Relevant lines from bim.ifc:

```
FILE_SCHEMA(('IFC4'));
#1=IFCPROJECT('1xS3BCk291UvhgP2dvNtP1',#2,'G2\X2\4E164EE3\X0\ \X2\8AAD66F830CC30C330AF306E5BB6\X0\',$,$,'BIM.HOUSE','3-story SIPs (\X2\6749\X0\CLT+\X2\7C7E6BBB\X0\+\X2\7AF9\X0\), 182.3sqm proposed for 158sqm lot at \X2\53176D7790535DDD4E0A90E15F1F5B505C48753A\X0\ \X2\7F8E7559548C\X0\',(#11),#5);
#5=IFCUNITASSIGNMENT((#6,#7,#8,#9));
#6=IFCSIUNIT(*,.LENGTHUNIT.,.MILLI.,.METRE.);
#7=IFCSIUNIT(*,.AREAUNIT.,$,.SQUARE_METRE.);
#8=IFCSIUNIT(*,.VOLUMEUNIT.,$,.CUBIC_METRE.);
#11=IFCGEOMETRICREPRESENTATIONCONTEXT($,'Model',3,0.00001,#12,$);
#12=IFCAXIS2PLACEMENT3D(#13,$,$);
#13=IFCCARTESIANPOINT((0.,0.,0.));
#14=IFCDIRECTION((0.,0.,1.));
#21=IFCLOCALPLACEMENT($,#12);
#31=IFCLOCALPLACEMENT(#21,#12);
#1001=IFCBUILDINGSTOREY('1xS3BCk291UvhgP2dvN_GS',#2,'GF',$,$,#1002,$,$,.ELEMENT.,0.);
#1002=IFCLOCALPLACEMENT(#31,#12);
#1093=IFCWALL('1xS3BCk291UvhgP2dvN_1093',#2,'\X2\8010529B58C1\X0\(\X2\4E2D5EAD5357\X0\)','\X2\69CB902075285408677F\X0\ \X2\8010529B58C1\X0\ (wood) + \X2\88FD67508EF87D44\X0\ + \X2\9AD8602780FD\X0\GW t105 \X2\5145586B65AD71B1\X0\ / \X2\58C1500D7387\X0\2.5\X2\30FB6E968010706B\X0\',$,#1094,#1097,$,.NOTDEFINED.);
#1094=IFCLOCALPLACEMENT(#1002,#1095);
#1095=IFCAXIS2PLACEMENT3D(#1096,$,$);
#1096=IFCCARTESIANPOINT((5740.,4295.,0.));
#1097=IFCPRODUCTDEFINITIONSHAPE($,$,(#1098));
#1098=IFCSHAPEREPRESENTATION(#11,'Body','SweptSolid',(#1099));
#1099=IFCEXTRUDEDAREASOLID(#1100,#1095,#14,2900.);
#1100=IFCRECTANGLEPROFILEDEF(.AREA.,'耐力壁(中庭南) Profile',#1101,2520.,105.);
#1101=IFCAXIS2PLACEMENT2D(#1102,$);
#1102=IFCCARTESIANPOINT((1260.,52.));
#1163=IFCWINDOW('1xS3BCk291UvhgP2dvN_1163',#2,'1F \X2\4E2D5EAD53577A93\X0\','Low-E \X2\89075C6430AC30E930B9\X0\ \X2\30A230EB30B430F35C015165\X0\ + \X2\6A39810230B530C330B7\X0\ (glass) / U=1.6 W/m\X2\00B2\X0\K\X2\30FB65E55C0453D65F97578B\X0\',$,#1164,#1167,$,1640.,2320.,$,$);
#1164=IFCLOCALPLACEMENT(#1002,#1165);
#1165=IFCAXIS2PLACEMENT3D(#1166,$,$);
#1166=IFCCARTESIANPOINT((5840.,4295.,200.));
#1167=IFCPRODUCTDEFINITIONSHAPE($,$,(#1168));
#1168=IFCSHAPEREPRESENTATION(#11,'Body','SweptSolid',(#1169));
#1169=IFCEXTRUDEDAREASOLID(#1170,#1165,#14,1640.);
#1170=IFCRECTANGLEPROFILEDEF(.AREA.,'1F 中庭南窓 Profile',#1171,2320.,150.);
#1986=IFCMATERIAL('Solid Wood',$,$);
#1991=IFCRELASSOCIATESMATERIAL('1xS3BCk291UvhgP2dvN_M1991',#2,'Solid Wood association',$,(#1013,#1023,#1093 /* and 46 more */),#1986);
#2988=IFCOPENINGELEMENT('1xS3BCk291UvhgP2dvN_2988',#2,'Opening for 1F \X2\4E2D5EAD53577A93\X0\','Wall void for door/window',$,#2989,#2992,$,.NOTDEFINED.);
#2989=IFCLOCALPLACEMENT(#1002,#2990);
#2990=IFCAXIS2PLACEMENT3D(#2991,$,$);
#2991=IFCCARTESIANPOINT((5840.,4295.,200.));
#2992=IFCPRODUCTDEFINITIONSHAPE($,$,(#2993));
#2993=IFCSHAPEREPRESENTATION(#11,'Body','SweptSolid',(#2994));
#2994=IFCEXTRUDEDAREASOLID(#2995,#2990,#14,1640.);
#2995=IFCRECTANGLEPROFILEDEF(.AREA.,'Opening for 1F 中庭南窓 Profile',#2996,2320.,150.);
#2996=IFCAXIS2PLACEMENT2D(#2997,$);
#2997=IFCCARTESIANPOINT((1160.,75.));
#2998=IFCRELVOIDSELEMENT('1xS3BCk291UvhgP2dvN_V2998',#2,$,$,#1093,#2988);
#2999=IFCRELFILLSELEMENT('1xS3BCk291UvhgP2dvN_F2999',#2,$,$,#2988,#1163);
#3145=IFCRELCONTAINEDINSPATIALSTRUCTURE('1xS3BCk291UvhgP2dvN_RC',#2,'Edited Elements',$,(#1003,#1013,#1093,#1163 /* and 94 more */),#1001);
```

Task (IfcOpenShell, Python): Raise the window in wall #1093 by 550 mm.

```python
import numpy as np
import ifcopenshell
import ifcopenshell.api.geometry
import ifcopenshell.util.placement
import ifcopenshell.util.unit

model = ifcopenshell.open("bim.ifc")
unit_scale = ifcopenshell.util.unit.calculate_unit_scale(model)

window = model.by_id(1163)
opening = window.FillsVoids[0].RelatingOpeningElement
dz = 550.0

shift = np.array([0.0, 0.0, dz])
# The window is not placed relative to its opening, so move both.
for product in (opening, window):
    matrix = ifcopenshell.util.placement.get_local_placement(product.ObjectPlacement)
    matrix[:3, 3] += shift
    ifcopenshell.api.geometry.edit_object_placement(model, product=product, matrix=matrix, is_si=False)

print(f"moved by {dz * unit_scale:+.3f} m")

model.write("bim_rev.ifc")
```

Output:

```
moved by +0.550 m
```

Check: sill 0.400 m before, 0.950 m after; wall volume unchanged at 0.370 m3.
